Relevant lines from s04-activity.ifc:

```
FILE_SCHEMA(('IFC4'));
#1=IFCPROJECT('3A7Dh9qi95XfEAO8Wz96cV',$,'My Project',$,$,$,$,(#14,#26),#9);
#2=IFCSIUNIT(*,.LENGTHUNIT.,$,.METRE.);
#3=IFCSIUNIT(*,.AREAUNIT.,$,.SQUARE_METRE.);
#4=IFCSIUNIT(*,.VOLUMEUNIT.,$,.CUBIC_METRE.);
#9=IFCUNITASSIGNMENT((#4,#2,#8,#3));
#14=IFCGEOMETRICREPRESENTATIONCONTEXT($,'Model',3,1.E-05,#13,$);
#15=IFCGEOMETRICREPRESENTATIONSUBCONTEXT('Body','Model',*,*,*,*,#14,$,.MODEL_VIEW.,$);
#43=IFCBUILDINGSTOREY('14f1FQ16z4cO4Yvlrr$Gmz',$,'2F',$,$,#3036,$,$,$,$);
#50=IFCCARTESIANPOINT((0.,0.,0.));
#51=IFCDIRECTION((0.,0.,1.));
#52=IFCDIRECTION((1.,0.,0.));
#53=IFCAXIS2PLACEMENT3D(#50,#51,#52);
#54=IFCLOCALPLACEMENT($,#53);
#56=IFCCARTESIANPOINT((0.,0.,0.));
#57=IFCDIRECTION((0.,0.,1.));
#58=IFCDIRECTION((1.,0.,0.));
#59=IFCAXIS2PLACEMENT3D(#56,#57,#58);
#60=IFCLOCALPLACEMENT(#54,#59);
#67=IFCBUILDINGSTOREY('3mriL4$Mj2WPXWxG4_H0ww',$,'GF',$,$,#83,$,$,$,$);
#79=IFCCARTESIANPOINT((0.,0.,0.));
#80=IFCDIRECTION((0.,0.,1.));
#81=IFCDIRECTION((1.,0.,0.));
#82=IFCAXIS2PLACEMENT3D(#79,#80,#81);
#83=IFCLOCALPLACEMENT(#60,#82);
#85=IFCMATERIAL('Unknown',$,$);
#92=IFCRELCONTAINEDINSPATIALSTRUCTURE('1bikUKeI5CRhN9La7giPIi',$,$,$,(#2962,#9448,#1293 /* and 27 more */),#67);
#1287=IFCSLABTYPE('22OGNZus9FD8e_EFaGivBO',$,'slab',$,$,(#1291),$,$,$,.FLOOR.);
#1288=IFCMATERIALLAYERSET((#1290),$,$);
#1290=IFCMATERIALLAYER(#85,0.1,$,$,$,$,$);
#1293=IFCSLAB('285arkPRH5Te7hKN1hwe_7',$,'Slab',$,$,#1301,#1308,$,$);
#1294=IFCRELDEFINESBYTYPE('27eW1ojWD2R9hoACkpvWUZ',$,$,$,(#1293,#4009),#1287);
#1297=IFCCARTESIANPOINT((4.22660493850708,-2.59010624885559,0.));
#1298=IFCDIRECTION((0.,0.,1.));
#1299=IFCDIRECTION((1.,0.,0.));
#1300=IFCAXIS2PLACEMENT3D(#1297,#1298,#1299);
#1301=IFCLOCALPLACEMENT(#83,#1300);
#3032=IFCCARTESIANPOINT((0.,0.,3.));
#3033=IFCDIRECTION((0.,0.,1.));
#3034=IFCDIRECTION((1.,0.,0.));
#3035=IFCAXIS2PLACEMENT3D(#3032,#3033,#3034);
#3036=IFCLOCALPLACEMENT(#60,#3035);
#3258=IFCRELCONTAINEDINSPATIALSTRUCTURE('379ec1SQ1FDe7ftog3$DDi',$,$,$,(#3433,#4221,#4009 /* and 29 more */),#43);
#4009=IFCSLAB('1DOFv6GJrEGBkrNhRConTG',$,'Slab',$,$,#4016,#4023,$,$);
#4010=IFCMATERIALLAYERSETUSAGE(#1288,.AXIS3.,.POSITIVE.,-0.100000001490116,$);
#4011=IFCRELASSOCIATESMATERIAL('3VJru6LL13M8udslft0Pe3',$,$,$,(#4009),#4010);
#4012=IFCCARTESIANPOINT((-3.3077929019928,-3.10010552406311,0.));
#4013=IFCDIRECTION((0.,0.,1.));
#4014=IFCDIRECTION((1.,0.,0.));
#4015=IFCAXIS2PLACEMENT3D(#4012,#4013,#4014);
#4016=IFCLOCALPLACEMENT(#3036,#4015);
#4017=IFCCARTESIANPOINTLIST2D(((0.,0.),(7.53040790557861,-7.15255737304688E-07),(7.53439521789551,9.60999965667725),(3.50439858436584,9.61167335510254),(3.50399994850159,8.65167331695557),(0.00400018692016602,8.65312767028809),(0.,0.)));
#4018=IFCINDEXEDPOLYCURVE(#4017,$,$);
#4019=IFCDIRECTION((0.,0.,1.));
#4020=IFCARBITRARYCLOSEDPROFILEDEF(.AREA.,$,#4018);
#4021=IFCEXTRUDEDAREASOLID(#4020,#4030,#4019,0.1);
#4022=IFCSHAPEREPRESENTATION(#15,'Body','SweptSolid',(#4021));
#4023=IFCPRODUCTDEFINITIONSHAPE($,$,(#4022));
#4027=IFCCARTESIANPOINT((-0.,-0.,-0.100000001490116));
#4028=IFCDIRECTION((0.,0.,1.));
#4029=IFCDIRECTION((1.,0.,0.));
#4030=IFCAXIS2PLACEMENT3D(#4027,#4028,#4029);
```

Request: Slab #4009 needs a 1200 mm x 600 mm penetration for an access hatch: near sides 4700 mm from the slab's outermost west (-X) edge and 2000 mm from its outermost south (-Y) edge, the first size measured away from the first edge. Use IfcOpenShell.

```python
import numpy as np
import ifcopenshell
import ifcopenshell.api.feature
import ifcopenshell.api.geometry
import ifcopenshell.api.root
import ifcopenshell.geom
import ifcopenshell.util.placement
import ifcopenshell.util.representation
import ifcopenshell.util.shape
import ifcopenshell.util.unit

model = ifcopenshell.open("s04-activity.ifc")
unit_scale = ifcopenshell.util.unit.calculate_unit_scale(model)
settings = ifcopenshell.geom.settings()


def volume(element):
    """Net volume in cubic metres, openings subtracted."""
    shape = ifcopenshell.geom.create_shape(settings, element)
    return ifcopenshell.util.shape.get_volume(shape.geometry)


slab = model.by_guid("1DOFv6GJrEGBkrNhRConTG")
before = volume(slab)

# Extent in the slab's own axes, in metres. The edges named are its -X and -Y sides.
slab_shape = ifcopenshell.geom.create_shape(settings, slab)
vertices = ifcopenshell.util.shape.get_vertices(slab_shape.geometry)
x_min, y_min, bottom = vertices.min(axis=0)
top = vertices[:, 2].max()

opening = ifcopenshell.api.root.create_entity(model, ifc_class="IfcOpeningElement", name="Access hatch opening", predefined_type="OPENING")
context = ifcopenshell.util.representation.get_context(model, "Model", "Body", "MODEL_VIEW")
width, depth = 1.2, 0.6
outline = [(0.0, 0.0), (width, 0.0), (width, depth), (0.0, depth), (0.0, 0.0)]
# Overshoot both faces by 50 mm so the cut is clean.
shape = ifcopenshell.api.geometry.add_slab_representation(
    model, context=context, depth=top - bottom + 0.1, polyline=outline
)
ifcopenshell.api.geometry.assign_representation(model, product=opening, representation=shape)

matrix = ifcopenshell.util.placement.get_local_placement(slab.ObjectPlacement)
matrix[:, 3] = matrix @ np.append(np.array([x_min + 4.7, y_min + 2, bottom - 0.05]) / unit_scale, 1.0)
ifcopenshell.api.geometry.edit_object_placement(model, product=opening, matrix=matrix, is_si=False)
ifcopenshell.api.feature.add_feature(model, feature=opening, element=slab)

after = volume(slab)

print(f"slab volume {before:.3f} -> {after:.3f} m3")

model.write("s04-activity-out.ifc")
```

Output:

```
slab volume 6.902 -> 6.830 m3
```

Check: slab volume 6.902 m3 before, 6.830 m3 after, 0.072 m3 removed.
